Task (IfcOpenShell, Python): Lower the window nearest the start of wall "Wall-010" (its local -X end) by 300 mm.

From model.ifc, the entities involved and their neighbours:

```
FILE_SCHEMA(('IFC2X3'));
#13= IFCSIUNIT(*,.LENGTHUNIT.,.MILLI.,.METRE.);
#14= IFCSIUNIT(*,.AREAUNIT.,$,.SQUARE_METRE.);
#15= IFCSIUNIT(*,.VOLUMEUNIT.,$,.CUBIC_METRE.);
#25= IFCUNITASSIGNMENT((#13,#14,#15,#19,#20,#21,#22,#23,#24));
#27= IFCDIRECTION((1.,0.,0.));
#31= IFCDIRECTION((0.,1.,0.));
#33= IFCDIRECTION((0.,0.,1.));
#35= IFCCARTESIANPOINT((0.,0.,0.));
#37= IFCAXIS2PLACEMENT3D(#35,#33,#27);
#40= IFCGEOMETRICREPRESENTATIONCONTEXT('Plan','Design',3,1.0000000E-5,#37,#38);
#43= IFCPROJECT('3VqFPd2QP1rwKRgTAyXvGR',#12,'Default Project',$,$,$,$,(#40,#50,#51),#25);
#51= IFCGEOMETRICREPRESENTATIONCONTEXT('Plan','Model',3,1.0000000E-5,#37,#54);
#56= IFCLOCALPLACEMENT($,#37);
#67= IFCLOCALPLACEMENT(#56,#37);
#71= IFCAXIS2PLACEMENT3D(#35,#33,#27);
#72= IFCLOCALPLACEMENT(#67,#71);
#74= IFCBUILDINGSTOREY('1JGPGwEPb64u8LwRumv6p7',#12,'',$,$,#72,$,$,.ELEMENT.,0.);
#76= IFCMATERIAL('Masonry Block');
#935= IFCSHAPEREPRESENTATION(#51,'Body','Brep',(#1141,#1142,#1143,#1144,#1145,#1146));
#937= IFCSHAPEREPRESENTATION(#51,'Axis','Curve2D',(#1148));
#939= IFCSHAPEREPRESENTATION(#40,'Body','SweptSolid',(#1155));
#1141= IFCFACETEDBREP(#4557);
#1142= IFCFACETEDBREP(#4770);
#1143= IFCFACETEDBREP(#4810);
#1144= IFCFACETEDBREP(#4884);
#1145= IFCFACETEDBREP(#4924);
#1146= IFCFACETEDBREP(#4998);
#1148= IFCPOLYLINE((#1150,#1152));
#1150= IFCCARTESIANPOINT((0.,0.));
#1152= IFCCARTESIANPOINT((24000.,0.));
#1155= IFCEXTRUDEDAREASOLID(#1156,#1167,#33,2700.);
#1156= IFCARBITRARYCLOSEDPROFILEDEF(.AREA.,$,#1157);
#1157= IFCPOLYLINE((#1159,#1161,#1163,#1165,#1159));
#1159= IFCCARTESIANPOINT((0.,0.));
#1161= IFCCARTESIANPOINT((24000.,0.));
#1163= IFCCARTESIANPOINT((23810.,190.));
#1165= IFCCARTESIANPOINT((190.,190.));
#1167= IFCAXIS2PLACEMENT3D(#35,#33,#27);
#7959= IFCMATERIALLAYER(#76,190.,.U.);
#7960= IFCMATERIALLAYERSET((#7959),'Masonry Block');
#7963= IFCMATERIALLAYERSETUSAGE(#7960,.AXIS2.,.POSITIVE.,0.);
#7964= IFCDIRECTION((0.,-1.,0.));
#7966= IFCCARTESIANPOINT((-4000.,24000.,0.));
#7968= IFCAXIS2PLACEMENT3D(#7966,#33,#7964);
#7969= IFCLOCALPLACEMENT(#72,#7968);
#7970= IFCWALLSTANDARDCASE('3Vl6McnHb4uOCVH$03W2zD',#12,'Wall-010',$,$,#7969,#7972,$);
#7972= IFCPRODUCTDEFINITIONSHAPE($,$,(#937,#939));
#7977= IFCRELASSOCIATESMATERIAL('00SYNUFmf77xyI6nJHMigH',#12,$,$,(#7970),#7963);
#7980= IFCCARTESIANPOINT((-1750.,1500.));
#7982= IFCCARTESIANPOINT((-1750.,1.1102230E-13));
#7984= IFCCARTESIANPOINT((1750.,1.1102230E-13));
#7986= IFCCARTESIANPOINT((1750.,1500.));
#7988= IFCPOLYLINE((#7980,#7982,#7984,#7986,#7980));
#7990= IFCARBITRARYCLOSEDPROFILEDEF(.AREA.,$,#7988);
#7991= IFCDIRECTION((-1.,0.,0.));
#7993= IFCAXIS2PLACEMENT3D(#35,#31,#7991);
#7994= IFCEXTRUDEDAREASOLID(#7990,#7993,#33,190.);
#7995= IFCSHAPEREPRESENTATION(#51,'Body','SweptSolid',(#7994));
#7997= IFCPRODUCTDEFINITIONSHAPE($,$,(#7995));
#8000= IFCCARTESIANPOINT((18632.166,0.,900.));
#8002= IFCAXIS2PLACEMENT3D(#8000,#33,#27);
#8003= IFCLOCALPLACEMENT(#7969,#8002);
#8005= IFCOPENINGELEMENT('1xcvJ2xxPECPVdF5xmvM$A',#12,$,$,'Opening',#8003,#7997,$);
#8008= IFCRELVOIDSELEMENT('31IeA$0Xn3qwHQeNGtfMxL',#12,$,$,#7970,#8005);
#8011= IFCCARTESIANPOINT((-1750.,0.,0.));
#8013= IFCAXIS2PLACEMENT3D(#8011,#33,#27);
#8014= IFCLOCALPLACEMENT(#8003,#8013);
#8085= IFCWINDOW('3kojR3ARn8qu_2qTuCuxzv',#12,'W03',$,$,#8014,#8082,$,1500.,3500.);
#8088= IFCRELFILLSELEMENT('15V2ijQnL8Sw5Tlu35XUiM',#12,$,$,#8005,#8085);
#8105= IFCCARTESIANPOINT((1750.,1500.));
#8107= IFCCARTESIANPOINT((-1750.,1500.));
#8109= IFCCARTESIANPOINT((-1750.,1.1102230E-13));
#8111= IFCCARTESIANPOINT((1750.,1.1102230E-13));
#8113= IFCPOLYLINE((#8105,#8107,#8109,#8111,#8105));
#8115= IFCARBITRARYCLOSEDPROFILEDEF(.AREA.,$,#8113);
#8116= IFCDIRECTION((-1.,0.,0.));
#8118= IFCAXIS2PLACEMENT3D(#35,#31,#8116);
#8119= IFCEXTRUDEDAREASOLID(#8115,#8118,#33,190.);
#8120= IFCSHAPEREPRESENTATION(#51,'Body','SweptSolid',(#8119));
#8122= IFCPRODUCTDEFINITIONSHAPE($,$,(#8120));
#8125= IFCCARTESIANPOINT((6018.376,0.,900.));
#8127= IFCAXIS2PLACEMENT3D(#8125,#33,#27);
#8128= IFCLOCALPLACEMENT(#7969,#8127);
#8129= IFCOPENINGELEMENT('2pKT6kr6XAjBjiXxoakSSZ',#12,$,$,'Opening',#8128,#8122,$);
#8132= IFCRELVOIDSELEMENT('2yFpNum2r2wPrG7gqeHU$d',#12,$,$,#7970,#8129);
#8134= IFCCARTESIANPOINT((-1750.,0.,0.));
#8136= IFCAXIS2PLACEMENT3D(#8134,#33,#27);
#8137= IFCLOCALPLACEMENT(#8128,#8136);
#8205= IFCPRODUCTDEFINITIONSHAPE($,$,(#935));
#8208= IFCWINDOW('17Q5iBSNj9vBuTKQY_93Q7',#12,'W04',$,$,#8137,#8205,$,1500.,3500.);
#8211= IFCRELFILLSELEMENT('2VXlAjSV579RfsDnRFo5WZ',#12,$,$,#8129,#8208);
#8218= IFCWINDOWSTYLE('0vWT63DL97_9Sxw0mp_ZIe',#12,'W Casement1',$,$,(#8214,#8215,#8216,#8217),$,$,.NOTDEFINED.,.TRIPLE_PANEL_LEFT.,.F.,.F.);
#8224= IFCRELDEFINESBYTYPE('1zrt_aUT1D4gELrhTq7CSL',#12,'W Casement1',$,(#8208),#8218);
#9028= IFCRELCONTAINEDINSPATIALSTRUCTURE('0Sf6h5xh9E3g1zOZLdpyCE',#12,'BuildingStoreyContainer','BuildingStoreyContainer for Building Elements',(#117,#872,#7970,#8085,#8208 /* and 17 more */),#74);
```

```python
import numpy as np
import ifcopenshell
import ifcopenshell.api.geometry
import ifcopenshell.util.placement
import ifcopenshell.util.unit

model = ifcopenshell.open("model.ifc")
unit_scale = ifcopenshell.util.unit.calculate_unit_scale(model)

window = model.by_guid("17Q5iBSNj9vBuTKQY_93Q7")
opening = window.FillsVoids[0].RelatingOpeningElement
dz = -0.3 / unit_scale

shift = np.array([0.0, 0.0, dz])
# The window is placed relative to its opening, so it follows when the opening moves.
matrix = ifcopenshell.util.placement.get_local_placement(opening.ObjectPlacement)
matrix[:3, 3] += shift
ifcopenshell.api.geometry.edit_object_placement(
    model, product=opening, matrix=matrix, is_si=False, should_transform_children=True
)

print(f"moved by {dz * unit_scale:+.3f} m")

model.write("model_v2.ifc")
```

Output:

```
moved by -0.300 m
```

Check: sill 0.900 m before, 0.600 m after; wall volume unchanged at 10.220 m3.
